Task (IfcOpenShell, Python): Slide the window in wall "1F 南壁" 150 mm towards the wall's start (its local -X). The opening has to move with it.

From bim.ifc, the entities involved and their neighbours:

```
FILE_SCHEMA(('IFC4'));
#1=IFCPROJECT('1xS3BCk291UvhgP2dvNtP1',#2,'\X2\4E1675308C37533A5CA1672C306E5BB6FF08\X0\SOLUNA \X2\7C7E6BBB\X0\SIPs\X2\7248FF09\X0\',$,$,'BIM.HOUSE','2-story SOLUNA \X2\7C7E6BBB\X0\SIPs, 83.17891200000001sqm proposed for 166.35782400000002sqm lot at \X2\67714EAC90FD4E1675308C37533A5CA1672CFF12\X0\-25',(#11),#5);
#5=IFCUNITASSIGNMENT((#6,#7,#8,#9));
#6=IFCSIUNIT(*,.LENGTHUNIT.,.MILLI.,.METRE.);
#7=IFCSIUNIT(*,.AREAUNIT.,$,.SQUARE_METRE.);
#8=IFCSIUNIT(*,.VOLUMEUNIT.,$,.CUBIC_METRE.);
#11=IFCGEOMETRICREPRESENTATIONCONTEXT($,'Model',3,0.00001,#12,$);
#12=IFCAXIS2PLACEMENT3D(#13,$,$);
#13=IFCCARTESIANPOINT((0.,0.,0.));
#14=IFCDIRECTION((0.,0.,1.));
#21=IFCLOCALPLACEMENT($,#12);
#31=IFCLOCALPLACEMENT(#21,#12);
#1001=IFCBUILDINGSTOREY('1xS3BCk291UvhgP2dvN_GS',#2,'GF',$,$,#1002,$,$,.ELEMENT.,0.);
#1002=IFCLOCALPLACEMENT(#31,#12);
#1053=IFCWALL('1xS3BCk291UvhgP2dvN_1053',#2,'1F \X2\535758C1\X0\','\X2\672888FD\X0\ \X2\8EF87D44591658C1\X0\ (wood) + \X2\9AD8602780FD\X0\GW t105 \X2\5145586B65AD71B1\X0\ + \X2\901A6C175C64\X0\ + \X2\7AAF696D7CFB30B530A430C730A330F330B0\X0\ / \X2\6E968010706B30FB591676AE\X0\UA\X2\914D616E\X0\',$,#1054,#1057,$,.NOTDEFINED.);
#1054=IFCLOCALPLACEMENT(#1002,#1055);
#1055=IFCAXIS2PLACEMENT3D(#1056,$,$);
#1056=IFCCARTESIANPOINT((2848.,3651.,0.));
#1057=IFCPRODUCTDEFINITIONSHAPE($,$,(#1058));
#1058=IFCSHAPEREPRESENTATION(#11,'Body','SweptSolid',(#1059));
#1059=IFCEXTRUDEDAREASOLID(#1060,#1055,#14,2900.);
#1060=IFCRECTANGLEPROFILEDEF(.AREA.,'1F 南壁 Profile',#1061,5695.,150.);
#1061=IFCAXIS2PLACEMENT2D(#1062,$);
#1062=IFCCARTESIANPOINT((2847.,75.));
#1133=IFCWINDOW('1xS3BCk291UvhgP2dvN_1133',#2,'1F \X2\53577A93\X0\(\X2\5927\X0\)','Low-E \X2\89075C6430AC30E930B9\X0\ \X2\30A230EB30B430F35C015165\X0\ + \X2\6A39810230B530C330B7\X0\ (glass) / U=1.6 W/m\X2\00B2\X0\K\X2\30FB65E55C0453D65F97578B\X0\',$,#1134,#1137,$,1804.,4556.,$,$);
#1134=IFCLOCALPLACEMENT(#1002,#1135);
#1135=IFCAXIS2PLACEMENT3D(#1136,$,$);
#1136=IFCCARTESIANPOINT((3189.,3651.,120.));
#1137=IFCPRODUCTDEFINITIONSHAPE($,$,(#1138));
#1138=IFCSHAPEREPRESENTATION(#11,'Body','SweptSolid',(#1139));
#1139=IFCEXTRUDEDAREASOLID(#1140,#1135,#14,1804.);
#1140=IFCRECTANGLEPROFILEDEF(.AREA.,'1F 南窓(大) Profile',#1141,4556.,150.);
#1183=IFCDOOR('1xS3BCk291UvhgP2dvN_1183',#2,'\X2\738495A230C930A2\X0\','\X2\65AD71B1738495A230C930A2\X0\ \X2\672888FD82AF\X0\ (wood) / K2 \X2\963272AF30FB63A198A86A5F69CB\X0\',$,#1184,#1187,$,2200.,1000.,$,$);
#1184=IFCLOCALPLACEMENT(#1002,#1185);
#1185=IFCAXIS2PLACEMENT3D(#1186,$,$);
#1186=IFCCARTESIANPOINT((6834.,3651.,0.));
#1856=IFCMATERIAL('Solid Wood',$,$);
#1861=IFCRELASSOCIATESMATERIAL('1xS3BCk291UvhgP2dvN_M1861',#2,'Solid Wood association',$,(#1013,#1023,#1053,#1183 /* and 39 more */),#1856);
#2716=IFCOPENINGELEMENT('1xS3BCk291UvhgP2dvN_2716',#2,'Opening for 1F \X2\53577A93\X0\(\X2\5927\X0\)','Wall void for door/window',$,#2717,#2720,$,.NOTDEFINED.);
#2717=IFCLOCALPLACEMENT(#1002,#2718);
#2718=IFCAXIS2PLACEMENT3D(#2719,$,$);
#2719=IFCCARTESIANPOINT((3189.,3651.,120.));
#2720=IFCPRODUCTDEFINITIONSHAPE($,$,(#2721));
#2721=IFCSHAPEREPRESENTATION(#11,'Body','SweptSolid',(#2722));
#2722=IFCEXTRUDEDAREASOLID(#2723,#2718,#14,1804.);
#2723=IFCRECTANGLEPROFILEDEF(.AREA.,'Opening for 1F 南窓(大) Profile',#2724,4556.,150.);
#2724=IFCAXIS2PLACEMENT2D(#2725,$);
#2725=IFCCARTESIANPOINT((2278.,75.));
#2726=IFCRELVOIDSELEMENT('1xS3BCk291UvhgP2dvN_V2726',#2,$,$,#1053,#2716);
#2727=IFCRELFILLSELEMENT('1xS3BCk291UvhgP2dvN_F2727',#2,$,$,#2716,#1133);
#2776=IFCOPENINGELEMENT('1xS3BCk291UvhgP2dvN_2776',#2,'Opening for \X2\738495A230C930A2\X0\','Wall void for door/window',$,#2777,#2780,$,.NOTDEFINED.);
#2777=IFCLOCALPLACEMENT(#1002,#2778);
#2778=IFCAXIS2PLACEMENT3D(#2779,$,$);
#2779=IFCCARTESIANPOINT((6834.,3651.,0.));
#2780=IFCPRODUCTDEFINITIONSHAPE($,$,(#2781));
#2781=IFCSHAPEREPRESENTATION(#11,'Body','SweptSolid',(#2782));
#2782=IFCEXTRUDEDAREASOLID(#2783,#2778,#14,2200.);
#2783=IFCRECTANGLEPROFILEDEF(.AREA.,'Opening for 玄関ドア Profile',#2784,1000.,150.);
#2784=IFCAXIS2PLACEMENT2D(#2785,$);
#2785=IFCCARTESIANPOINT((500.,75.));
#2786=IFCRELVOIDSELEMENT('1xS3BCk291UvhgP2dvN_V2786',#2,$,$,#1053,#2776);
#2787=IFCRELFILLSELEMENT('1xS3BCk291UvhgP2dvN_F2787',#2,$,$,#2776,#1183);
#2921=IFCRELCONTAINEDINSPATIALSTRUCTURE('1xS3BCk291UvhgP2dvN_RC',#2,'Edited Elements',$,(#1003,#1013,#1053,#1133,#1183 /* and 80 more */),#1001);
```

```python
import ifcopenshell
import ifcopenshell.api.geometry
import ifcopenshell.util.placement
import ifcopenshell.util.unit

model = ifcopenshell.open("bim.ifc")
unit_scale = ifcopenshell.util.unit.calculate_unit_scale(model)

window = model.by_id(1133)
opening = window.FillsVoids[0].RelatingOpeningElement
wall = opening.VoidsElements[0].RelatingBuildingElement

wall_matrix = ifcopenshell.util.placement.get_local_placement(wall.ObjectPlacement)
shift = wall_matrix[:3, 0] * -0.15 / unit_scale
before = ifcopenshell.util.placement.get_local_placement(window.ObjectPlacement)[:3, 3].copy()

# The window is not placed relative to its opening, so move both.
for product in (opening, window):
    matrix = ifcopenshell.util.placement.get_local_placement(product.ObjectPlacement)
    matrix[:3, 3] += shift
    ifcopenshell.api.geometry.edit_object_placement(model, product=product, matrix=matrix, is_si=False)

after = ifcopenshell.util.placement.get_local_placement(window.ObjectPlacement)[:3, 3]
print("window moved by", (after - before).round(3) + 0.0)

model.write("bim-out.ifc")
```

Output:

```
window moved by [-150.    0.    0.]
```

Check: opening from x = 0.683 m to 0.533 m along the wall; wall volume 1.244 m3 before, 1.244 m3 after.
